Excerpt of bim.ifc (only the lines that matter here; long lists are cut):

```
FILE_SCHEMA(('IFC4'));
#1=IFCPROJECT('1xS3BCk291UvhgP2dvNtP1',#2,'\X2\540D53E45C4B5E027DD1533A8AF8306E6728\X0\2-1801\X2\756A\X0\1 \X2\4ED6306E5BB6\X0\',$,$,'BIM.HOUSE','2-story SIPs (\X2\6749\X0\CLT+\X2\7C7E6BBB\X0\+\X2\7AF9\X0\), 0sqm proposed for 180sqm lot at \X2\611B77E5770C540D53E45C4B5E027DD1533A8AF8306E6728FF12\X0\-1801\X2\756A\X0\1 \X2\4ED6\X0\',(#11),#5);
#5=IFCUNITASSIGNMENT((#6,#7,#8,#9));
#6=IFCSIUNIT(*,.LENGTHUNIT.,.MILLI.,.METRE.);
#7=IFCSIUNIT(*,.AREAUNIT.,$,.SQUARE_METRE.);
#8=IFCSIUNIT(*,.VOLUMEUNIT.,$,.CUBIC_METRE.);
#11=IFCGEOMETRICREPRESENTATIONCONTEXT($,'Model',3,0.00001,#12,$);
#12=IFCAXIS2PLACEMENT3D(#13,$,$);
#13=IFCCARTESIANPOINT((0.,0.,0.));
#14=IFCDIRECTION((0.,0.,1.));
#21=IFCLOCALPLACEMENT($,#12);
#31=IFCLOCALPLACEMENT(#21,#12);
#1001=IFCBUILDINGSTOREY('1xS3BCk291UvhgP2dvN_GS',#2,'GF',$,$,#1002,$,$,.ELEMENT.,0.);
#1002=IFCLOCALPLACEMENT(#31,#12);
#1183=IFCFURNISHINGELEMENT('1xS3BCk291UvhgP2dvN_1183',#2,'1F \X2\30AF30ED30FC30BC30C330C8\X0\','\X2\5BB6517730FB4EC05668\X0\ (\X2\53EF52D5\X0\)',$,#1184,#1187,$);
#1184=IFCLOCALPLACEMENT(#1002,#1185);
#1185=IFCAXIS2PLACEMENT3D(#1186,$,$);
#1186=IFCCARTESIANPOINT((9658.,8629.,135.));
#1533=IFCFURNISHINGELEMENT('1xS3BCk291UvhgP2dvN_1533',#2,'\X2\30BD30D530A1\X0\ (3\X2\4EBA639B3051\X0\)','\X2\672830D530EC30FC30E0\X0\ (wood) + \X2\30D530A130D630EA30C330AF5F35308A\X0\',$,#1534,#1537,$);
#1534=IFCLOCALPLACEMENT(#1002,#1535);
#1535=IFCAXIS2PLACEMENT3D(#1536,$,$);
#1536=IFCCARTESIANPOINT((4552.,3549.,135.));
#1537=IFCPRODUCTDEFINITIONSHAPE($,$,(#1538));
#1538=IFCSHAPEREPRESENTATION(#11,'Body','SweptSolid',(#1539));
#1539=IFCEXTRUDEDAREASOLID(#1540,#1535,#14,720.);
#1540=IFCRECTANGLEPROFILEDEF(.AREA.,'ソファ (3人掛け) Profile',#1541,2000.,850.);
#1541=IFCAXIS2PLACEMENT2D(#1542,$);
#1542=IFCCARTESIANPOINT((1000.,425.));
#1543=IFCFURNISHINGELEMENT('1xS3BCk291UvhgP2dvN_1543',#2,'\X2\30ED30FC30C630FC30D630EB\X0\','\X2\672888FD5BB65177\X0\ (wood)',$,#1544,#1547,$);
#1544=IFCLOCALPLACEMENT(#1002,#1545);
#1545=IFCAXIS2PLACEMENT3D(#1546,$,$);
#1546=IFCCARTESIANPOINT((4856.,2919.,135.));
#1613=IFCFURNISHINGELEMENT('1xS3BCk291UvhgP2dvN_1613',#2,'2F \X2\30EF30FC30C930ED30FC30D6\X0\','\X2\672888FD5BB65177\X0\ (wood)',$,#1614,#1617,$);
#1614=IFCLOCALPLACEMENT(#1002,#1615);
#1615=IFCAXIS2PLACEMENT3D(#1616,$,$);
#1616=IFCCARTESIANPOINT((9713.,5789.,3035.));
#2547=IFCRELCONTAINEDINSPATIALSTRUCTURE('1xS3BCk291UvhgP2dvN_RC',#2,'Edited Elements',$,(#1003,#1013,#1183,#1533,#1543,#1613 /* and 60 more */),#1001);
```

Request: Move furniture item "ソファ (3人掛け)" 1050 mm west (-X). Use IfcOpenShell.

```python
import ifcopenshell
import ifcopenshell.api.geometry
import ifcopenshell.util.placement
import ifcopenshell.util.unit

model = ifcopenshell.open("bim.ifc")
unit_scale = ifcopenshell.util.unit.calculate_unit_scale(model)

item = model.by_id(1533)
matrix = ifcopenshell.util.placement.get_local_placement(item.ObjectPlacement)
matrix[0, 3] -= 1.05 / unit_scale
ifcopenshell.api.geometry.edit_object_placement(model, product=item, matrix=matrix, is_si=False)

print(ifcopenshell.util.placement.get_local_placement(item.ObjectPlacement).round(3) + 0.0)

model.write("bim_rev.ifc")
```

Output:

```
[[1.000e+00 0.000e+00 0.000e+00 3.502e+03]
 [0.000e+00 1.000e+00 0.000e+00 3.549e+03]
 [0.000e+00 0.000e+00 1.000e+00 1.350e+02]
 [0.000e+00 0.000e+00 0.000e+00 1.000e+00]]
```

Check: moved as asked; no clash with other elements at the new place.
